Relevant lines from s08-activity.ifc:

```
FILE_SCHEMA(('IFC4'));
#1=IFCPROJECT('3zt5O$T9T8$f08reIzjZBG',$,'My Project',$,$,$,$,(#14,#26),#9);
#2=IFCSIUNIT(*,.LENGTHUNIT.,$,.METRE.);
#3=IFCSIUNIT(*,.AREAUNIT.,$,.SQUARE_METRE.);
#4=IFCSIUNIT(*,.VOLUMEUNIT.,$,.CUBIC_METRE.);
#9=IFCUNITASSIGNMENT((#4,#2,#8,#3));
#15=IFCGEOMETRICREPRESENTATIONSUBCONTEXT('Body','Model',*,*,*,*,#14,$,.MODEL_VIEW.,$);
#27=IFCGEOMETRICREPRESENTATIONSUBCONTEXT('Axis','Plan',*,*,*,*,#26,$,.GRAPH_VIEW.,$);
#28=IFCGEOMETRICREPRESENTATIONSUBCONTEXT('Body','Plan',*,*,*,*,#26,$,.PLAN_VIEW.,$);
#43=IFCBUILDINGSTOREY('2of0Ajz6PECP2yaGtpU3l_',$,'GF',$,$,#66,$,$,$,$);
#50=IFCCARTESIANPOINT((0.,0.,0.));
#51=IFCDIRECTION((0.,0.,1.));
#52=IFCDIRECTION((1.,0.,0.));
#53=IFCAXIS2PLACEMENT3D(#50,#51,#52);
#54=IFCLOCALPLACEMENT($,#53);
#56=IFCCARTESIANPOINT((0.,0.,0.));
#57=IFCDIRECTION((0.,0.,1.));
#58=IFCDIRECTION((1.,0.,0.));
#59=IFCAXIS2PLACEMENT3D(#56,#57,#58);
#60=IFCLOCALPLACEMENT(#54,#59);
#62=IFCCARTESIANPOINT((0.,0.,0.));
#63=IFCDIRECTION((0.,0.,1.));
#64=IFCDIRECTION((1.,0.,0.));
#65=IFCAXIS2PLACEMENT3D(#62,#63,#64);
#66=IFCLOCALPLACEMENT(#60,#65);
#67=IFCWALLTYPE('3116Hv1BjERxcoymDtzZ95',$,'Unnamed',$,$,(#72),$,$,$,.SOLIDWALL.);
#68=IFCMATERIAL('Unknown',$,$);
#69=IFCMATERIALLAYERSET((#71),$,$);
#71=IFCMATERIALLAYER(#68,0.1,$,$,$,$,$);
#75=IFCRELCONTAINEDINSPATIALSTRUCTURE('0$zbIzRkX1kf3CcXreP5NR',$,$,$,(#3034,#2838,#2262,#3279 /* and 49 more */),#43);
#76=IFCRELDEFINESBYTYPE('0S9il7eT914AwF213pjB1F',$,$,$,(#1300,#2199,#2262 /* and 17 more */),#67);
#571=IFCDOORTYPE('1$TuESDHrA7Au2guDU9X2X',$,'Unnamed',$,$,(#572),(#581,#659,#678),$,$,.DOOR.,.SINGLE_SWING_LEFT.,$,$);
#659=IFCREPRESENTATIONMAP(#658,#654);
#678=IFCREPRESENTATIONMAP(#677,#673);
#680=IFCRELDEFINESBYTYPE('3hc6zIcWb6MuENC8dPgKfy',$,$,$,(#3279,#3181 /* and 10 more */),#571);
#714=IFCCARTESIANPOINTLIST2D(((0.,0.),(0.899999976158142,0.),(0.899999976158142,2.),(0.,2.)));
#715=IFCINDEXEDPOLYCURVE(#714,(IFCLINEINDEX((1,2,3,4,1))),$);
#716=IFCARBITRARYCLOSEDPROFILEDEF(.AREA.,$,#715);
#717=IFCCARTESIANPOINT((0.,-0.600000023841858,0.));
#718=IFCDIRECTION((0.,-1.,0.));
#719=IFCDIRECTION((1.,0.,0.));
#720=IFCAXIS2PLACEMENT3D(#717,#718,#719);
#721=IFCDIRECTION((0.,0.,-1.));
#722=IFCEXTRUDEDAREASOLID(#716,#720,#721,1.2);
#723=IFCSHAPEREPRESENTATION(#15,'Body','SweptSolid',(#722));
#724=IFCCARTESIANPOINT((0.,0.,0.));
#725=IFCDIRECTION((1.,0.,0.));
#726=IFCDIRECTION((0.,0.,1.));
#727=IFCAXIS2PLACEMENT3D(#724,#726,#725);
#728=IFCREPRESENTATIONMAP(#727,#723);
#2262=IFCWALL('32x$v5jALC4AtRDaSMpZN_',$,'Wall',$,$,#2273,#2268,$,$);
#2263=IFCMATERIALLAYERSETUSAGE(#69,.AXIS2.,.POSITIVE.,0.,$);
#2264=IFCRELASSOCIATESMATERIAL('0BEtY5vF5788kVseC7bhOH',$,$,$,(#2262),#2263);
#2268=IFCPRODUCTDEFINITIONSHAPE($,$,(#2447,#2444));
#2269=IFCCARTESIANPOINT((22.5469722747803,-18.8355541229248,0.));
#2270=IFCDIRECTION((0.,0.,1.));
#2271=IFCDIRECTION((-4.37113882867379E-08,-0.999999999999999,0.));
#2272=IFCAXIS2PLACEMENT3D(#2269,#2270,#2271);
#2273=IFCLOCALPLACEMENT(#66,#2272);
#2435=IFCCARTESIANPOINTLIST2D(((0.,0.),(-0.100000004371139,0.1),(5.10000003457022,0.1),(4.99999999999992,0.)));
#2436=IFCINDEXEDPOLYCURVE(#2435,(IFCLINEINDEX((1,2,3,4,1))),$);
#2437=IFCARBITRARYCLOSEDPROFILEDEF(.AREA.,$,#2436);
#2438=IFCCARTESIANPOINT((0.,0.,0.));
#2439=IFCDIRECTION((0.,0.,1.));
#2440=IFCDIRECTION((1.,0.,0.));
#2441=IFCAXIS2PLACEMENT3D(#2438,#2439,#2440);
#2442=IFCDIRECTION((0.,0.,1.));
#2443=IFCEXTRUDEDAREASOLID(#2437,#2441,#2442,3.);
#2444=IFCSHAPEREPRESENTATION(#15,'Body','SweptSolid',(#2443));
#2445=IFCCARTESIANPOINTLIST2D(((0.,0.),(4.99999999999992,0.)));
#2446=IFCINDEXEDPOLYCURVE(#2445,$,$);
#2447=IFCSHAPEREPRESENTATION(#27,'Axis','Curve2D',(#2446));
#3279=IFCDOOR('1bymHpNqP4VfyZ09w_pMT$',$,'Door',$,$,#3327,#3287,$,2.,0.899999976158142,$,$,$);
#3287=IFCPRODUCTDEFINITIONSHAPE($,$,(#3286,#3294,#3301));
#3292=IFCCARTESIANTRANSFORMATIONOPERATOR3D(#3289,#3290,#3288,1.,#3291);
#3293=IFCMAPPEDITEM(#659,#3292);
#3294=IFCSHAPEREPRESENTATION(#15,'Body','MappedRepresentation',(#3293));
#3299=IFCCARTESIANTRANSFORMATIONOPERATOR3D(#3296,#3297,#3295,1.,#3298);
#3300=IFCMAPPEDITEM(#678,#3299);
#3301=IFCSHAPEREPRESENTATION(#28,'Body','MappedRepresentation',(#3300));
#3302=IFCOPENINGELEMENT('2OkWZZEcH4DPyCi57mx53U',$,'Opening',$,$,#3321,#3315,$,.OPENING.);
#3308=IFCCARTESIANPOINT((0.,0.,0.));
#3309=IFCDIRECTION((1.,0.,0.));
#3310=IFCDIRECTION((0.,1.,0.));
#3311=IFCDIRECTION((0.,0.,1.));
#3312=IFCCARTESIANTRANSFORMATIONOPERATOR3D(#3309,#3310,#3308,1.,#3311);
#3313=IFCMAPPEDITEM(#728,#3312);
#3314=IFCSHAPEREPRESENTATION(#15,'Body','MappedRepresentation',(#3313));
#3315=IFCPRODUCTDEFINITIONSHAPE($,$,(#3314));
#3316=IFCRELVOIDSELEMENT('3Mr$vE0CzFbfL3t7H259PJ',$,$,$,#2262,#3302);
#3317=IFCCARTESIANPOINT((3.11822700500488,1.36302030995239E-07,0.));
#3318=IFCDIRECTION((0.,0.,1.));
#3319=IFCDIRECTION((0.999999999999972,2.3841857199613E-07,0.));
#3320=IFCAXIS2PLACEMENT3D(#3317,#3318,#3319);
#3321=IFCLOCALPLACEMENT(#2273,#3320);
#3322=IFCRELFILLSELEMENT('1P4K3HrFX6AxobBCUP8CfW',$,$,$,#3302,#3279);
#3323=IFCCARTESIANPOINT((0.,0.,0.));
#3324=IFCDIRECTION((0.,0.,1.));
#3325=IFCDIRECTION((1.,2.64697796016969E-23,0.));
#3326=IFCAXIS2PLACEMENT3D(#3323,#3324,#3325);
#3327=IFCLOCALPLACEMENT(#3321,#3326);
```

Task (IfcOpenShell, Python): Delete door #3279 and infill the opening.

```python
import ifcopenshell
import ifcopenshell.api.feature
import ifcopenshell.api.root
import ifcopenshell.geom
import ifcopenshell.util.shape

model = ifcopenshell.open("s08-activity.ifc")
settings = ifcopenshell.geom.settings()


def volume(element):
    """Net volume in cubic metres, openings subtracted."""
    shape = ifcopenshell.geom.create_shape(settings, element)
    return ifcopenshell.util.shape.get_volume(shape.geometry)


door = model.by_guid("1bymHpNqP4VfyZ09w_pMT$")
opening = door.FillsVoids[0].RelatingOpeningElement
wall = opening.VoidsElements[0].RelatingBuildingElement
before = volume(wall)

ifcopenshell.api.root.remove_product(model, product=door)
ifcopenshell.api.feature.remove_feature(model, feature=opening)

after = volume(wall)

print(f"wall volume {before:.3f} -> {after:.3f} m3")

model.write("s08-activity_v2.ifc")
```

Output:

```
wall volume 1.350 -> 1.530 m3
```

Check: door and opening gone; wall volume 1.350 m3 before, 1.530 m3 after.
